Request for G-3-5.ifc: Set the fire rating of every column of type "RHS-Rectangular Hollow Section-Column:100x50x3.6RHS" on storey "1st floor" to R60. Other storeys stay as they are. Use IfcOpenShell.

First a look at what the model holds.

```python
import ifcopenshell
import ifcopenshell.util.element

model = ifcopenshell.open("G-3-5.ifc")
print(model.schema)
storey = next(s for s in model.by_type("IfcBuildingStorey") if s.Name == "1st floor")
columns = [e for e in ifcopenshell.util.element.get_decomposition(storey) if e.is_a("IfcColumn")]
seen = {}
for e in columns:
    element_type = ifcopenshell.util.element.get_type(e)
    key = (element_type.Name if element_type != e and element_type else None, ifcopenshell.util.element.get_pset(e, "Pset_ColumnCommon", "FireRating"))
    seen[key] = seen.get(key, 0) + 1
for (name, value), count in sorted(seen.items(), key=str):
    print(count, "x", name, "|", value)
```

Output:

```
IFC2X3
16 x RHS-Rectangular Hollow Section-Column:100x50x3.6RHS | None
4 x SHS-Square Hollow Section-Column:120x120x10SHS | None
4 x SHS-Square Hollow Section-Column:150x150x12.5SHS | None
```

```python
import ifcopenshell
import ifcopenshell.api.pset
import ifcopenshell.util.element

model = ifcopenshell.open("G-3-5.ifc")

storey = next(s for s in model.by_type("IfcBuildingStorey") if s.Name == "1st floor")
columns = [e for e in ifcopenshell.util.element.get_decomposition(storey) if e.is_a("IfcColumn")]

count = 0
for e in columns:
    element_type = ifcopenshell.util.element.get_type(e)
    if element_type in (None, e) or element_type.Name != "RHS-Rectangular Hollow Section-Column:100x50x3.6RHS":
        continue
    # add_pset returns the element's existing set when there is one.
    pset = ifcopenshell.api.pset.add_pset(model, product=e, name="Pset_ColumnCommon")
    ifcopenshell.api.pset.edit_pset(model, pset=pset, properties={"FireRating": "R60"})
    count += 1

print(count, "columns updated")

model.write("G-3-5_rev.ifc")
```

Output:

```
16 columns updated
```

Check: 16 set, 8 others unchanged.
